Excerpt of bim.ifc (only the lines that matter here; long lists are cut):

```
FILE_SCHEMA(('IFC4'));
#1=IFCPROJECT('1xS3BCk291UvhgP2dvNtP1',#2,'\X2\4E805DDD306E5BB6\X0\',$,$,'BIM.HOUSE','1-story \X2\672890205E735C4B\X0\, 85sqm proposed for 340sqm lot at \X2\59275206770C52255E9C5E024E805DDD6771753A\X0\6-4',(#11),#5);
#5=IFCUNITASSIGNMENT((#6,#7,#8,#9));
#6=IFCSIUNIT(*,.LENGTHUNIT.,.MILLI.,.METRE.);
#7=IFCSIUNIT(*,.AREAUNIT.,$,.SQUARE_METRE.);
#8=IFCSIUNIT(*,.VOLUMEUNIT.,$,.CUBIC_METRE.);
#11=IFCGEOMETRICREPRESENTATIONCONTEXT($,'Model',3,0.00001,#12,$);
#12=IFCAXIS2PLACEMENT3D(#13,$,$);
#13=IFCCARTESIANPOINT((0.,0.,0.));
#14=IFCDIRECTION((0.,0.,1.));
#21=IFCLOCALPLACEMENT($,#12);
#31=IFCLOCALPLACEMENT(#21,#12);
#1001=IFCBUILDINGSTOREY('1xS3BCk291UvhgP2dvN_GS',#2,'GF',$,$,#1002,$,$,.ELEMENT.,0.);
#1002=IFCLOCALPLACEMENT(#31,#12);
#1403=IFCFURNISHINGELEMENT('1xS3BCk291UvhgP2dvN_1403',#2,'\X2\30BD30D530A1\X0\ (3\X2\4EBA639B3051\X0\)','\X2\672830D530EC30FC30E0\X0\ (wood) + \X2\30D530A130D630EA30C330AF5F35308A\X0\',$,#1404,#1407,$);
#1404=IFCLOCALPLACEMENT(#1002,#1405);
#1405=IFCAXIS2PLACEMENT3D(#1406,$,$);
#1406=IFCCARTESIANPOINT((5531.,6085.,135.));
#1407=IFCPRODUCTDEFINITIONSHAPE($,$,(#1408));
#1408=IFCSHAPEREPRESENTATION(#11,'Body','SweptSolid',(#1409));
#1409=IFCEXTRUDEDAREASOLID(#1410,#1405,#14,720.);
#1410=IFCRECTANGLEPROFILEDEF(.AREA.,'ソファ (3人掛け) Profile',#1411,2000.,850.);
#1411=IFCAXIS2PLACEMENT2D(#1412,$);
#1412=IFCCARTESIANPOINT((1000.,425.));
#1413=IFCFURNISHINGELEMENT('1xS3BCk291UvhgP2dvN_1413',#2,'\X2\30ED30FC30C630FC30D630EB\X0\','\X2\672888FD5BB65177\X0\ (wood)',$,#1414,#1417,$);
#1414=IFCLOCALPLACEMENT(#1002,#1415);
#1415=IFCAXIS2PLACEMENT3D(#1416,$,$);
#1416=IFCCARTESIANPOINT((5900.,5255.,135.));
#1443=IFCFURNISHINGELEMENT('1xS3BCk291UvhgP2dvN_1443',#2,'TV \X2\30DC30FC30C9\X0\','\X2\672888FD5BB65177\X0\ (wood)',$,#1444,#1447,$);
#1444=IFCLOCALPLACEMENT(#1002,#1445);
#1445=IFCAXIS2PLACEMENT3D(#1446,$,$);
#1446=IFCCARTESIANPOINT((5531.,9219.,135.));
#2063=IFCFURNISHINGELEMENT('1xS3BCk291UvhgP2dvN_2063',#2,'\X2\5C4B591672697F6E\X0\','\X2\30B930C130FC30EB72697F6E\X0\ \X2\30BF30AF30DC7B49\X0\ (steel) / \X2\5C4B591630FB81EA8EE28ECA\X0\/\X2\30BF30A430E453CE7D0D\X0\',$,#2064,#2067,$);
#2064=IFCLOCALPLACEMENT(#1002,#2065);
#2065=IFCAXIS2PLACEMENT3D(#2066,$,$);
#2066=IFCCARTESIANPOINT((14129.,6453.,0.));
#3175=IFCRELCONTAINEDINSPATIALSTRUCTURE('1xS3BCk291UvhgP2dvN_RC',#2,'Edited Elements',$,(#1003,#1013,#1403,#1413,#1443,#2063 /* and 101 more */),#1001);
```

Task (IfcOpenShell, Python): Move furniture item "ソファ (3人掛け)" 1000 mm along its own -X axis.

```python
import ifcopenshell
import ifcopenshell.api.geometry
import ifcopenshell.util.placement
import ifcopenshell.util.unit

model = ifcopenshell.open("bim.ifc")
unit_scale = ifcopenshell.util.unit.calculate_unit_scale(model)

item = model.by_id(1403)
matrix = ifcopenshell.util.placement.get_local_placement(item.ObjectPlacement)
matrix[:3, 3] -= matrix[:3, 0] * 1 / unit_scale
ifcopenshell.api.geometry.edit_object_placement(model, product=item, matrix=matrix, is_si=False)

print(ifcopenshell.util.placement.get_local_placement(item.ObjectPlacement).round(3) + 0.0)

model.write("bim_v2.ifc")
```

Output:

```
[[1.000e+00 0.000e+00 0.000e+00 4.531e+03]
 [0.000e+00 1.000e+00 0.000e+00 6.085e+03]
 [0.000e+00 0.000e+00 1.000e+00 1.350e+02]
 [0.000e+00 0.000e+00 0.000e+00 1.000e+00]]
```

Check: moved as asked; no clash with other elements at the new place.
